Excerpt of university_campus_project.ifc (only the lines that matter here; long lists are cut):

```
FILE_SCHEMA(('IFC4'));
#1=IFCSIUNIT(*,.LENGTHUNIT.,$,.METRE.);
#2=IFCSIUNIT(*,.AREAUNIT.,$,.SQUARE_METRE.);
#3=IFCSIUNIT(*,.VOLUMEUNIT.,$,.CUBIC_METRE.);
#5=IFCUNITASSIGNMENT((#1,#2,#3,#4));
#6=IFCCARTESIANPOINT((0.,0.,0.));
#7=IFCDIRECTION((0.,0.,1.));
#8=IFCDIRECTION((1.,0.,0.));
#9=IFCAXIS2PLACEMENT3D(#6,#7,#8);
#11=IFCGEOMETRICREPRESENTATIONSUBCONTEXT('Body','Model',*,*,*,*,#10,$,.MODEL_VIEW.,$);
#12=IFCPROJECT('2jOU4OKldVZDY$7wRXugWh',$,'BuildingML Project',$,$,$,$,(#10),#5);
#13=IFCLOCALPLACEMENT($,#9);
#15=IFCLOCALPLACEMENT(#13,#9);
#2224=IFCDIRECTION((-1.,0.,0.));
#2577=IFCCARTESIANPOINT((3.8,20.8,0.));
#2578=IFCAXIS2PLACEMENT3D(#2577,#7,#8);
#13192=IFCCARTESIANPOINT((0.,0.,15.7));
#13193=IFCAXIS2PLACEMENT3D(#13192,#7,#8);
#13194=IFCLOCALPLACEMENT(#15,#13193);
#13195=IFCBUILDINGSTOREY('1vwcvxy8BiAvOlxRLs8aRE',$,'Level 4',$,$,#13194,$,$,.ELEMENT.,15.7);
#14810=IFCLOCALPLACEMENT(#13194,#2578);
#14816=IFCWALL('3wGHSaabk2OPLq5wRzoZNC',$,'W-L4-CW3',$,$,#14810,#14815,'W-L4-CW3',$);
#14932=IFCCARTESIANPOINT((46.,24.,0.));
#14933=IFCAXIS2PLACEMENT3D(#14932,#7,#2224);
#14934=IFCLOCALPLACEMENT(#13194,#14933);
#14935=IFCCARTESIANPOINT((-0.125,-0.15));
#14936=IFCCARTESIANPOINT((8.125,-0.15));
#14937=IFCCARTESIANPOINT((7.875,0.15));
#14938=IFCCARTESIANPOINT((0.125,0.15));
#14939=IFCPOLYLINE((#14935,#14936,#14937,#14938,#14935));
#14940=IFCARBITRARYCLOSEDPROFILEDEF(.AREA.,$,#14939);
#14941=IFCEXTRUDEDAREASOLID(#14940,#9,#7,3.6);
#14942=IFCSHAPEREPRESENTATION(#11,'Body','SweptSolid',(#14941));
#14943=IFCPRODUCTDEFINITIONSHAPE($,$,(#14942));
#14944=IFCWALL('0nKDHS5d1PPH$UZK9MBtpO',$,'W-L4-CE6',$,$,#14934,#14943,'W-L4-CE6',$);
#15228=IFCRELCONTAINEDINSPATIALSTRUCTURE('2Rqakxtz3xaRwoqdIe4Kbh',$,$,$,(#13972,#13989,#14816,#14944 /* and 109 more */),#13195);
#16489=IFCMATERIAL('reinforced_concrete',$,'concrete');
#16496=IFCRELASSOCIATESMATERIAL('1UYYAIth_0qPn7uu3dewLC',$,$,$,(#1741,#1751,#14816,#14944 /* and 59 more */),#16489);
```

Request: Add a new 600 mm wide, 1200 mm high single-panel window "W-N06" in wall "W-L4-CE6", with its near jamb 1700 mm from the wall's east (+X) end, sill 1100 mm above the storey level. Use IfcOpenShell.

```python
import numpy as np
import ifcopenshell
import ifcopenshell.api.feature
import ifcopenshell.api.geometry
import ifcopenshell.api.root
import ifcopenshell.api.spatial
import ifcopenshell.geom
import ifcopenshell.util.element
import ifcopenshell.util.placement
import ifcopenshell.util.representation
import ifcopenshell.util.shape
import ifcopenshell.util.unit

model = ifcopenshell.open("university_campus_project.ifc")
unit_scale = ifcopenshell.util.unit.calculate_unit_scale(model)
settings = ifcopenshell.geom.settings()


def volume(element):
    """Net volume in cubic metres, openings subtracted."""
    shape = ifcopenshell.geom.create_shape(settings, element)
    return ifcopenshell.util.shape.get_volume(shape.geometry)


wall = model.by_id(14944)
storey = ifcopenshell.util.element.get_container(wall, ifc_class="IfcBuildingStorey")
context = ifcopenshell.util.representation.get_context(model, "Model", "Body", "MODEL_VIEW")
before = volume(wall)

width, height, from_end, sill = 0.6, 1.2, 1.7, 1.1  # metres

# The wall runs along its own X axis, and the end named is its -X end.
wall_shape = ifcopenshell.geom.create_shape(settings, wall)
x, y, z = ifcopenshell.util.shape.get_vertices(wall_shape.geometry).T
start = x.min() + from_end
face, thickness = float(y.min()), float(y.max() - y.min())
wall_matrix = ifcopenshell.util.placement.get_local_placement(wall.ObjectPlacement)
level = ifcopenshell.util.placement.get_local_placement(storey.ObjectPlacement)[2, 3]


def in_wall(x, y):
    """Placement at x, y metres in the wall's axes, at sill height."""
    matrix = wall_matrix.copy()
    matrix[:, 3] = wall_matrix @ np.array([x / unit_scale, y / unit_scale, 0.0, 1.0])
    matrix[2, 3] = level + sill / unit_scale
    return matrix


# Opening: a box that overshoots both wall faces by 50 mm.
opening = ifcopenshell.api.root.create_entity(model, ifc_class="IfcOpeningElement", predefined_type="OPENING")
box = ifcopenshell.api.geometry.add_wall_representation(
    model, context=context, length=width, height=height, thickness=thickness + 0.1
)
ifcopenshell.api.geometry.assign_representation(model, product=opening, representation=box)
ifcopenshell.api.geometry.edit_object_placement(model, product=opening, matrix=in_wall(start, face - 0.05), is_si=False)
ifcopenshell.api.feature.add_feature(model, feature=opening, element=wall)

window = ifcopenshell.api.root.create_entity(model, ifc_class="IfcWindow", name="W-N06", predefined_type="WINDOW")
window.OverallWidth, window.OverallHeight = width / unit_scale, height / unit_scale
window.PartitioningType = "SINGLE_PANEL"
body = ifcopenshell.api.geometry.add_window_representation(
    model,
    context=context,
    overall_width=window.OverallWidth,
    overall_height=window.OverallHeight,
    partition_type="SINGLE_PANEL",
)
ifcopenshell.api.geometry.assign_representation(model, product=window, representation=body)
ifcopenshell.api.spatial.assign_container(model, products=[window], relating_structure=storey)
ifcopenshell.api.feature.add_filling(model, opening=opening, element=window)

# Centre the window in the wall's thickness.
ifcopenshell.api.geometry.edit_object_placement(model, product=window, matrix=in_wall(start, face), is_si=False)
window_shape = ifcopenshell.geom.create_shape(settings, window)
depth = ifcopenshell.util.shape.get_vertices(window_shape.geometry)[:, 1]
offset = face + thickness / 2 - (depth.min() + depth.max()) / 2
ifcopenshell.api.geometry.edit_object_placement(model, product=window, matrix=in_wall(start, offset), is_si=False)

after = volume(wall)

print(f"wall volume {before:.3f} -> {after:.3f} m3")

model.write("university_campus_project_updated.ifc")
```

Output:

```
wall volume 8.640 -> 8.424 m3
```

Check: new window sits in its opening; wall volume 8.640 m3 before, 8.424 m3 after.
